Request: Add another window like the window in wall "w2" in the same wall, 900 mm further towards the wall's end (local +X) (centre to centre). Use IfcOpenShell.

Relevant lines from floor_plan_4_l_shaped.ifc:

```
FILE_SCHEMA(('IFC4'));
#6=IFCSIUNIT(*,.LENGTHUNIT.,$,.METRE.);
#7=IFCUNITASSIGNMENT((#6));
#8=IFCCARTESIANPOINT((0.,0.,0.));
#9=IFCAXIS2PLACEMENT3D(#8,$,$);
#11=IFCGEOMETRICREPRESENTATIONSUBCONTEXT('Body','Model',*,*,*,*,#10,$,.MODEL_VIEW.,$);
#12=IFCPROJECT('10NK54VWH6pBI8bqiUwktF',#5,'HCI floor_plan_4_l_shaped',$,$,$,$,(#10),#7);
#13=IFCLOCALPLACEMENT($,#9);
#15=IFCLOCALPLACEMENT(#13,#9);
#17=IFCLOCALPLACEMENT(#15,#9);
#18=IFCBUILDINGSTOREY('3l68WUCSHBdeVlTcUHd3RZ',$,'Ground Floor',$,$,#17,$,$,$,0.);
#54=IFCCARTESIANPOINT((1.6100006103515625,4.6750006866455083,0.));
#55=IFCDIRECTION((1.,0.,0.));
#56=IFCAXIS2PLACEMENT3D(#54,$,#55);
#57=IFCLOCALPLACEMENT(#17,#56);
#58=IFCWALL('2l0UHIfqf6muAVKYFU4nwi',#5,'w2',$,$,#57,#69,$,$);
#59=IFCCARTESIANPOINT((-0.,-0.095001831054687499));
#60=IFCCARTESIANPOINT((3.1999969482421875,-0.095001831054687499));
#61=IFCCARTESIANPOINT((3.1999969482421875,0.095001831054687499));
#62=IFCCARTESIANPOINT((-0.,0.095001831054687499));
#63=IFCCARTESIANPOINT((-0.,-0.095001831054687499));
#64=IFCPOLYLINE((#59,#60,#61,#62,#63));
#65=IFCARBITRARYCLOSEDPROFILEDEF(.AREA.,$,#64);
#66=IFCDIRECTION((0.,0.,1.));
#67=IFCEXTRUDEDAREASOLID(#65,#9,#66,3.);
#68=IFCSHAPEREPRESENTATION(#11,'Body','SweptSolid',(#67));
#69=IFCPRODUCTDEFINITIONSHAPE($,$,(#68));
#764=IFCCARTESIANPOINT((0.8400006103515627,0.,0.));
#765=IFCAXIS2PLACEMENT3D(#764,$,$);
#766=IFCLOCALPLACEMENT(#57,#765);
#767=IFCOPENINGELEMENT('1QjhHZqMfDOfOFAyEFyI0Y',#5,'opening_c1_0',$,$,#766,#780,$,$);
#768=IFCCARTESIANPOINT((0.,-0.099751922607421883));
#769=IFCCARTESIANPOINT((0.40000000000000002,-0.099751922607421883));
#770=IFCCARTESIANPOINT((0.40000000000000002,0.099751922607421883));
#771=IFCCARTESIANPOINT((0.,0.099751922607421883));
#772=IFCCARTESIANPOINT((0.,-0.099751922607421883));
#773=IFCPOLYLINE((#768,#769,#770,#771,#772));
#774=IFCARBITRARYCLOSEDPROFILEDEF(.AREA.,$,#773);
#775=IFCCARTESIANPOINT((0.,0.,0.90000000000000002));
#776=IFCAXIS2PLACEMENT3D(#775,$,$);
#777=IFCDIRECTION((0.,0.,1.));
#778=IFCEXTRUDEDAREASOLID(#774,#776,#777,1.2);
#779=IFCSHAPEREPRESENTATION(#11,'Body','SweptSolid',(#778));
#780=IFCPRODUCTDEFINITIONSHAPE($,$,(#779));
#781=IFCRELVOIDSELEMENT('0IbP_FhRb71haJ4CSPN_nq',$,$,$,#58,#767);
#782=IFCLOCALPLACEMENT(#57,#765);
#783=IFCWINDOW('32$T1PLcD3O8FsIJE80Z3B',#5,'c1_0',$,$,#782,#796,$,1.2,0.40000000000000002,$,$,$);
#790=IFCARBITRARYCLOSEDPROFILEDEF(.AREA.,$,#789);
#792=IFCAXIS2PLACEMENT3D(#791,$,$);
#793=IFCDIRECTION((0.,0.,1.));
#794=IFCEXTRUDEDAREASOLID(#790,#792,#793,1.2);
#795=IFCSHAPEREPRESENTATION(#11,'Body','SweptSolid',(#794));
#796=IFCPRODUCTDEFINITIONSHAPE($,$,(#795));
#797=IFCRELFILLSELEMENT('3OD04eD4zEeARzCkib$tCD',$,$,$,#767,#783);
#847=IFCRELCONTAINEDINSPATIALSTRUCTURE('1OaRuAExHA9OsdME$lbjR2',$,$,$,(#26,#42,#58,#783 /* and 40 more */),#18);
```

```python
import ifcopenshell
import ifcopenshell.api.feature
import ifcopenshell.api.geometry
import ifcopenshell.api.root
import ifcopenshell.geom
import ifcopenshell.util.element
import ifcopenshell.util.placement
import ifcopenshell.util.shape

model = ifcopenshell.open("floor_plan_4_l_shaped.ifc")
settings = ifcopenshell.geom.settings()


def volume(element):
    """Net volume in cubic metres, openings subtracted."""
    shape = ifcopenshell.geom.create_shape(settings, element)
    return ifcopenshell.util.shape.get_volume(shape.geometry)


window = model.by_guid("32$T1PLcD3O8FsIJE80Z3B")
opening = window.FillsVoids[0].RelatingOpeningElement
wall = opening.VoidsElements[0].RelatingBuildingElement
before = volume(wall)
shift = ifcopenshell.util.placement.get_local_placement(wall.ObjectPlacement)[:3, 0] * 0.9

# copy_class copies the void relationship, type, container and properties, but no geometry.
new_opening = ifcopenshell.api.root.copy_class(model, product=opening)
new_opening.Representation = ifcopenshell.util.element.copy_deep(
    model, opening.Representation, exclude=["IfcGeometricRepresentationContext", "IfcRepresentationMap"]
)
new_window = ifcopenshell.api.root.copy_class(model, product=window)
new_window.Representation = ifcopenshell.util.element.copy_deep(
    model, window.Representation, exclude=["IfcGeometricRepresentationContext", "IfcRepresentationMap"]
)
ifcopenshell.api.feature.add_filling(model, opening=new_opening, element=new_window)

for old, new in ((opening, new_opening), (window, new_window)):
    matrix = ifcopenshell.util.placement.get_local_placement(old.ObjectPlacement)
    matrix[:3, 3] += shift
    ifcopenshell.api.geometry.edit_object_placement(model, product=new, matrix=matrix, is_si=False)

after = volume(wall)

print(f"wall volume {before:.3f} -> {after:.3f} m3")

model.write("floor_plan_4_l_shaped_edited.ifc")
```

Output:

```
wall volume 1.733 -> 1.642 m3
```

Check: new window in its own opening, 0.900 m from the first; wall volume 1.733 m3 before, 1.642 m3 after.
